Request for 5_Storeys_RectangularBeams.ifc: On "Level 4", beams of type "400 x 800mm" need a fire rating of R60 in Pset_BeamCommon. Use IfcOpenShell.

First a look at what the model holds.

```python
import ifcopenshell
import ifcopenshell.util.element

model = ifcopenshell.open("5_Storeys_RectangularBeams.ifc")
print(model.schema)
storey = next(s for s in model.by_type("IfcBuildingStorey") if s.Name == "Level 4")
beams = [e for e in ifcopenshell.util.element.get_decomposition(storey) if e.is_a("IfcBeam")]
seen = {}
for e in beams:
    element_type = ifcopenshell.util.element.get_type(e)
    key = (element_type.Name if element_type != e and element_type else None, ifcopenshell.util.element.get_pset(e, "Pset_BeamCommon", "FireRating"))
    seen[key] = seen.get(key, 0) + 1
for (name, value), count in sorted(seen.items(), key=str):
    print(count, "x", name, "|", value)
```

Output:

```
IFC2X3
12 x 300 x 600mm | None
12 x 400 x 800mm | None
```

```python
import ifcopenshell
import ifcopenshell.api.pset
import ifcopenshell.util.element

model = ifcopenshell.open("5_Storeys_RectangularBeams.ifc")

storey = next(s for s in model.by_type("IfcBuildingStorey") if s.Name == "Level 4")
beams = [e for e in ifcopenshell.util.element.get_decomposition(storey) if e.is_a("IfcBeam")]

count = 0
for e in beams:
    element_type = ifcopenshell.util.element.get_type(e)
    if element_type in (None, e) or element_type.Name != "400 x 800mm":
        continue
    # add_pset returns the element's existing set when there is one.
    pset = ifcopenshell.api.pset.add_pset(model, product=e, name="Pset_BeamCommon")
    ifcopenshell.api.pset.edit_pset(model, pset=pset, properties={"FireRating": "R60"})
    count += 1

print(count, "beams updated")

model.write("5_Storeys_RectangularBeams_updated.ifc")
```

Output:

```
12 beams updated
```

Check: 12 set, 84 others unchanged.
